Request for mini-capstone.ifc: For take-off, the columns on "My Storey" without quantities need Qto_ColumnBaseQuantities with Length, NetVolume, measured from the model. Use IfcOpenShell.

First a look at what the model holds.

```python
import ifcopenshell
import ifcopenshell.util.element
import ifcopenshell.util.unit

model = ifcopenshell.open("mini-capstone.ifc")
print(model.schema)
for unit_type in ("LENGTHUNIT", "AREAUNIT", "VOLUMEUNIT"):
    print(unit_type, ifcopenshell.util.unit.calculate_unit_scale(model, unit_type))
storey = next(s for s in model.by_type("IfcBuildingStorey") if s.Name == "My Storey")
columns = [e for e in ifcopenshell.util.element.get_decomposition(storey) if e.is_a("IfcColumn")]
for e in sorted(columns, key=lambda e: e.id()):
    print(e.id(), e.is_a(), e.Name, list(ifcopenshell.util.element.get_psets(e, qtos_only=True)), sep=" | ")
```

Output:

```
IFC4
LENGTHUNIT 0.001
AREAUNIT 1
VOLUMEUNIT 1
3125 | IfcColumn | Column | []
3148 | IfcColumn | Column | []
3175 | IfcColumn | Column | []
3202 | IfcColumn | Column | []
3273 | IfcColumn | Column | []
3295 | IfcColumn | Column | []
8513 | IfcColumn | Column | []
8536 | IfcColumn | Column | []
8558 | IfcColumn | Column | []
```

```python
import ifcopenshell
import ifcopenshell.api.pset
import ifcopenshell.geom
import ifcopenshell.util.element
import ifcopenshell.util.shape
import ifcopenshell.util.unit

model = ifcopenshell.open("mini-capstone.ifc")
unit_scale = ifcopenshell.util.unit.calculate_unit_scale(model)
volume_scale = ifcopenshell.util.unit.calculate_unit_scale(model, "VOLUMEUNIT")
settings = ifcopenshell.geom.settings()

storey = next(s for s in model.by_type("IfcBuildingStorey") if s.Name == "My Storey")
columns = [e for e in ifcopenshell.util.element.get_decomposition(storey) if e.is_a("IfcColumn")]

for e in sorted(columns, key=lambda e: e.id()):
    if ifcopenshell.util.element.get_psets(e, qtos_only=True, should_inherit=False):
        continue
    # Geometry comes back in metres, in the element's own axes.
    shape = ifcopenshell.geom.create_shape(settings, e)
    values = {
        "Length": ifcopenshell.util.shape.get_z(shape.geometry) / unit_scale,
        "NetVolume": ifcopenshell.util.shape.get_volume(shape.geometry) / volume_scale,
    }
    qto = ifcopenshell.api.pset.add_qto(model, product=e, name="Qto_ColumnBaseQuantities")
    ifcopenshell.api.pset.edit_qto(model, qto=qto, properties=values)
    print(e.id(), {k: round(v, 3) for k, v in values.items()})

model.write("mini-capstone_updated.ifc")
```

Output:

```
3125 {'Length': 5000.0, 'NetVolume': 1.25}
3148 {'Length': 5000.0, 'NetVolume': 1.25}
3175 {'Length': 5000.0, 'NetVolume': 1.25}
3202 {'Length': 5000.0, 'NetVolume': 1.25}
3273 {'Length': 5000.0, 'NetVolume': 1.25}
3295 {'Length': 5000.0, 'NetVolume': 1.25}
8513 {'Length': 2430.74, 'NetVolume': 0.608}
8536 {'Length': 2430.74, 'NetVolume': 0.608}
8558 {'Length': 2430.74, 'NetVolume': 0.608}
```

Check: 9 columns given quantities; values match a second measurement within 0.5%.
